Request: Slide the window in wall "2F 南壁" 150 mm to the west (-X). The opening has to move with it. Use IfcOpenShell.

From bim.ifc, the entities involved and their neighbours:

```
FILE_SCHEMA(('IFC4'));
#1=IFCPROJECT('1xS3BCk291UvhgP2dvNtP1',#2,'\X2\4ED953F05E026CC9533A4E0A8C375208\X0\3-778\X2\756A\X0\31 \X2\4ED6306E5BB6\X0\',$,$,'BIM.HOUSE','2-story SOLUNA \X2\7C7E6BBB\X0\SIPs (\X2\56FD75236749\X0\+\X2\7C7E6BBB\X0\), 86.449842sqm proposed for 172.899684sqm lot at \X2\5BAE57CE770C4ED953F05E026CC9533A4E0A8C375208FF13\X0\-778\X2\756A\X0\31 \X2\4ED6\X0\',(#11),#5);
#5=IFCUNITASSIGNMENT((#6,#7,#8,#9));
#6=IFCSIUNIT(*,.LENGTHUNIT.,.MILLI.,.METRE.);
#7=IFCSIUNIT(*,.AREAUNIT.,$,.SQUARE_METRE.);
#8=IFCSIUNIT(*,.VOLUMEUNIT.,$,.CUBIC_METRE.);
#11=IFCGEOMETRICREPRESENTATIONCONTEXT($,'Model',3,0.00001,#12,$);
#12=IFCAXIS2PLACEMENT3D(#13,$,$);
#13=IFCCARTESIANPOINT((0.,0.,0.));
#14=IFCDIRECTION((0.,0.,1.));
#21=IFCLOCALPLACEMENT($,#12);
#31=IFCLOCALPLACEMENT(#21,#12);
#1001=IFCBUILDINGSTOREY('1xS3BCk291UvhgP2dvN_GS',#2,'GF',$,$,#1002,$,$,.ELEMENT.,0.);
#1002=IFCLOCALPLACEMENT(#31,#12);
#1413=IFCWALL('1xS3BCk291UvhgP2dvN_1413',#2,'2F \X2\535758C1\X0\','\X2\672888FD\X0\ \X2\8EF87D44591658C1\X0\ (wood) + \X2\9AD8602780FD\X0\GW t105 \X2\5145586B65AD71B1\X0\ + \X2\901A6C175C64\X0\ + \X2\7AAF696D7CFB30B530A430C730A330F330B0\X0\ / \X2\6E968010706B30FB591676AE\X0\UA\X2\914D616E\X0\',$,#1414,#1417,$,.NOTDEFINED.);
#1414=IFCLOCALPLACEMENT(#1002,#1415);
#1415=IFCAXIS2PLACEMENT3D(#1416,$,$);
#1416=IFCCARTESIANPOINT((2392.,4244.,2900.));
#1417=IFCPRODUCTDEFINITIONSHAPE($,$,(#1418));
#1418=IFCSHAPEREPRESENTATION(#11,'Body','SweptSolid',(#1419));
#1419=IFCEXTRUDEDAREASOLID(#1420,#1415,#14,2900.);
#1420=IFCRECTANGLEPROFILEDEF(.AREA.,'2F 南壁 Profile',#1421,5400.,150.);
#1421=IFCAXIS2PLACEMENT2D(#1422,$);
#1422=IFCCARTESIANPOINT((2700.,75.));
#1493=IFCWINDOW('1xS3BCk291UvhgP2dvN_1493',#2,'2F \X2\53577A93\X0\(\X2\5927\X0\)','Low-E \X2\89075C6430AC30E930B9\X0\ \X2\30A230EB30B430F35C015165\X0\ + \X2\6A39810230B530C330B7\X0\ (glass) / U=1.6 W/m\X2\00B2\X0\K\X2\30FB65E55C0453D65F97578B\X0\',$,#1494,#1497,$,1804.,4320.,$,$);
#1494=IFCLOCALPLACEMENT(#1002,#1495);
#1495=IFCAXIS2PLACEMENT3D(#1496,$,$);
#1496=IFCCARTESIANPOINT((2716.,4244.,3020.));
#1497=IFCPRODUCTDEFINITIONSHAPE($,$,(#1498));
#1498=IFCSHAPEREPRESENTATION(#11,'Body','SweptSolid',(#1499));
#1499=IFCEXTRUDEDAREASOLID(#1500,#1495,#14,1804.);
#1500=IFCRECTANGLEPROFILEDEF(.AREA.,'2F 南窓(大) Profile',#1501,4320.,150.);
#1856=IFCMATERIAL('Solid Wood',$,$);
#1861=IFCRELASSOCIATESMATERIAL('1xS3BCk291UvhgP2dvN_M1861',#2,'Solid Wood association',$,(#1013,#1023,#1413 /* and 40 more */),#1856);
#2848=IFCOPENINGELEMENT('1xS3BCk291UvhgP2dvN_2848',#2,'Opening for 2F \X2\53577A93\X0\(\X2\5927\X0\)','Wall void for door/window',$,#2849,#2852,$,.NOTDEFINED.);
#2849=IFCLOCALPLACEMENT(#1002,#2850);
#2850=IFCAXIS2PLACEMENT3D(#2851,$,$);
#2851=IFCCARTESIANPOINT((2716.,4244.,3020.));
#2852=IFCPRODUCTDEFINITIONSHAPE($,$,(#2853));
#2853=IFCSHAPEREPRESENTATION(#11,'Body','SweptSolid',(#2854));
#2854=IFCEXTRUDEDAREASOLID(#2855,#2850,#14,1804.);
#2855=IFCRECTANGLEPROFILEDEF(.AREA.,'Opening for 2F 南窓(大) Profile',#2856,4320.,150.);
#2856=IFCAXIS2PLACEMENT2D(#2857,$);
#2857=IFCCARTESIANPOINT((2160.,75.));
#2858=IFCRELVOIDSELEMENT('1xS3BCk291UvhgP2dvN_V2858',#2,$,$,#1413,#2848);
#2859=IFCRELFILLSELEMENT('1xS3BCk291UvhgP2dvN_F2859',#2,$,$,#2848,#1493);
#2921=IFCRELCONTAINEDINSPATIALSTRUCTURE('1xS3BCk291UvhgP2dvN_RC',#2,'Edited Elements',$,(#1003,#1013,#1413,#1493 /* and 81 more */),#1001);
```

```python
import ifcopenshell
import ifcopenshell.api.geometry
import ifcopenshell.util.placement
import ifcopenshell.util.unit

model = ifcopenshell.open("bim.ifc")
unit_scale = ifcopenshell.util.unit.calculate_unit_scale(model)

window = model.by_id(1493)
opening = window.FillsVoids[0].RelatingOpeningElement
wall = opening.VoidsElements[0].RelatingBuildingElement

wall_matrix = ifcopenshell.util.placement.get_local_placement(wall.ObjectPlacement)
shift = wall_matrix[:3, 0] * -0.15 / unit_scale
before = ifcopenshell.util.placement.get_local_placement(window.ObjectPlacement)[:3, 3].copy()

# The window is not placed relative to its opening, so move both.
for product in (opening, window):
    matrix = ifcopenshell.util.placement.get_local_placement(product.ObjectPlacement)
    matrix[:3, 3] += shift
    ifcopenshell.api.geometry.edit_object_placement(model, product=product, matrix=matrix, is_si=False)

after = ifcopenshell.util.placement.get_local_placement(window.ObjectPlacement)[:3, 3]
print("window moved by", (after - before).round(3) + 0.0)

model.write("bim-out.ifc")
```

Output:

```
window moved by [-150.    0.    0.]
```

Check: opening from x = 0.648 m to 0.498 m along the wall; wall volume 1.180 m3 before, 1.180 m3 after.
